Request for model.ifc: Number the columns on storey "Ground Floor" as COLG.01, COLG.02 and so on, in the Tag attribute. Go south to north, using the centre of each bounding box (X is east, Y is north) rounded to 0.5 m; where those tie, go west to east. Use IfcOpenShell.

First a look at what the model holds.

```python
import ifcopenshell
import ifcopenshell.util.element
import ifcopenshell.util.placement

model = ifcopenshell.open("model.ifc")
print(model.schema)
storey = next(s for s in model.by_type("IfcBuildingStorey") if s.Name == "Ground Floor")
columns = [e for e in ifcopenshell.util.element.get_decomposition(storey) if e.is_a("IfcColumn")]
for e in sorted(columns, key=lambda e: e.id()):
    origin = ifcopenshell.util.placement.get_local_placement(e.ObjectPlacement)[:3, 3]
    print(e.id(), e.Tag, e.Name, origin.round(2) + 0.0, sep=" | ")
```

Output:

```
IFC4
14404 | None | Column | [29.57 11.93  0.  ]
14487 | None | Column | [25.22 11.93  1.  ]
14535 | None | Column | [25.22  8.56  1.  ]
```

```python
import ifcopenshell
import ifcopenshell.geom
import ifcopenshell.util.element
import ifcopenshell.util.shape

model = ifcopenshell.open("model.ifc")
settings = ifcopenshell.geom.settings()
settings.set("use-world-coords", True)


def centre(element):
    shape = ifcopenshell.geom.create_shape(settings, element)
    return ifcopenshell.util.shape.get_bbox_centroid(shape.geometry)


storey = next(s for s in model.by_type("IfcBuildingStorey") if s.Name == "Ground Floor")
columns = [e for e in ifcopenshell.util.element.get_decomposition(storey) if e.is_a("IfcColumn")]

# Insertion points can sit at a corner or the storey origin, so sort by the geometry (in metres).
centres = {e: centre(e) for e in columns}
columns.sort(key=lambda e: (round(centres[e][1] / 0.5), centres[e][0]))

for i, e in enumerate(columns, start=1):
    number = f"COLG.{i:02d}"
    e.Tag = number
    print(e.id(), number)

model.write("model_edited.ifc")
```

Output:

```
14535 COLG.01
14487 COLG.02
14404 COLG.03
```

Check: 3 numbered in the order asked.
